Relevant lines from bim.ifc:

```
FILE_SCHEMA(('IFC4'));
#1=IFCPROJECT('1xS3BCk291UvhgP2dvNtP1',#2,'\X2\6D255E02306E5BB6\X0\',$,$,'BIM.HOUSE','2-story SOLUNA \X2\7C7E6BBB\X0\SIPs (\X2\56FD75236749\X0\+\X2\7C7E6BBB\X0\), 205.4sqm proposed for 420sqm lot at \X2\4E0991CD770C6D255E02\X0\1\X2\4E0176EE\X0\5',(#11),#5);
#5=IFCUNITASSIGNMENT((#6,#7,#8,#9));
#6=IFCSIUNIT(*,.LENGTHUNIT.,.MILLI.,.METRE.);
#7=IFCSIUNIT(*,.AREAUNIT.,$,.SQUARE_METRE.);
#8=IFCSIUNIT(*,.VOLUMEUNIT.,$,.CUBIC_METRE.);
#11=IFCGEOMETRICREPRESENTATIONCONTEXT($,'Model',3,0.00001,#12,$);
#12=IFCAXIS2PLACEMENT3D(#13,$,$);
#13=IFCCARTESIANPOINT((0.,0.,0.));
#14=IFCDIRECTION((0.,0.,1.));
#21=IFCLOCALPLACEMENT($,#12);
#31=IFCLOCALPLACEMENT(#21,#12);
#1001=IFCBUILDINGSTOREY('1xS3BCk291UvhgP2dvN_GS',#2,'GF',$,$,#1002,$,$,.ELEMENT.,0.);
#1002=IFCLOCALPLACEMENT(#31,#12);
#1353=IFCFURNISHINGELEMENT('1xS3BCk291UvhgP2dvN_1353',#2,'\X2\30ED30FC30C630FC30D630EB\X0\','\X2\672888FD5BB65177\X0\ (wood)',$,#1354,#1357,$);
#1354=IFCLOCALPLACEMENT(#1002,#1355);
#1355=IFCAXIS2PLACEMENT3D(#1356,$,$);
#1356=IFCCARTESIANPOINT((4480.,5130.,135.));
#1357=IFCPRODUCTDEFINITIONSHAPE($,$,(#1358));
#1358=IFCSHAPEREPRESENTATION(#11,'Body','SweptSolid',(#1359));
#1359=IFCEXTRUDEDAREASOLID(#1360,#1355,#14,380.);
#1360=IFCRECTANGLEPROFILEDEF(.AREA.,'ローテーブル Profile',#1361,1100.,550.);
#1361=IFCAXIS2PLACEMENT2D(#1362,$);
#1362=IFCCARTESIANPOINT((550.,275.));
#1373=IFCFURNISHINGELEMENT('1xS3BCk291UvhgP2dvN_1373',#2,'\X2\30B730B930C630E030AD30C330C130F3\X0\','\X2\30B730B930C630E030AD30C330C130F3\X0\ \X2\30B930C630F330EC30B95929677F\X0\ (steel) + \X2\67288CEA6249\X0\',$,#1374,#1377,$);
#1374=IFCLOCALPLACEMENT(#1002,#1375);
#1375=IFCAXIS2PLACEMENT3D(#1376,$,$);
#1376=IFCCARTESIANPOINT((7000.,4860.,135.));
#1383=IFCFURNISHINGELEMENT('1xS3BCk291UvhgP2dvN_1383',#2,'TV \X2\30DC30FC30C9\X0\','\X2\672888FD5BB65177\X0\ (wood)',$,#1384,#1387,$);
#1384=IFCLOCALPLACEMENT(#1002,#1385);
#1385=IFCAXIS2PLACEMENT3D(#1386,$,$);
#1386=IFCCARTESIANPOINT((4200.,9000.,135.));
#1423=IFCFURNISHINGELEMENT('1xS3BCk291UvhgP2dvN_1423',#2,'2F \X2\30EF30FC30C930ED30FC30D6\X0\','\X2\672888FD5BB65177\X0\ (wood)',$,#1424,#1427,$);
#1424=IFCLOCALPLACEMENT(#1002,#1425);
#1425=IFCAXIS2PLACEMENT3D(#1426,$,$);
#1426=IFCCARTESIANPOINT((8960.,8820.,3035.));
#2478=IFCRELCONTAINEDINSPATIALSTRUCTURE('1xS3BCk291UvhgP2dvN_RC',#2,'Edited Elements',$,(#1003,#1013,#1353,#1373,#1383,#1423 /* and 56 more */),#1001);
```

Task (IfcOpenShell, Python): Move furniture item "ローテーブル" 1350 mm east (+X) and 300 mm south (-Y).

```python
import ifcopenshell
import ifcopenshell.api.geometry
import ifcopenshell.util.placement
import ifcopenshell.util.unit

model = ifcopenshell.open("bim.ifc")
unit_scale = ifcopenshell.util.unit.calculate_unit_scale(model)

item = model.by_guid("1xS3BCk291UvhgP2dvN_1353")
matrix = ifcopenshell.util.placement.get_local_placement(item.ObjectPlacement)
matrix[0, 3] += 1.35 / unit_scale
matrix[1, 3] -= 0.3 / unit_scale
ifcopenshell.api.geometry.edit_object_placement(model, product=item, matrix=matrix, is_si=False)

print(ifcopenshell.util.placement.get_local_placement(item.ObjectPlacement).round(3) + 0.0)

model.write("bim_rev.ifc")
```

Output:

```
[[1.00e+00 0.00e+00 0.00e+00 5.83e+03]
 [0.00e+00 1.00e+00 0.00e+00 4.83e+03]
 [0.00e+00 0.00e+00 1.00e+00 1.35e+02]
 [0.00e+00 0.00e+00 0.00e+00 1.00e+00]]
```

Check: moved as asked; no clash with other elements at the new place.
